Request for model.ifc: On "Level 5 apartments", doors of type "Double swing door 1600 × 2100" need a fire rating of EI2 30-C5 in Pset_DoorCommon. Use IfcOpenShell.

First a look at what the model holds.

```python
import ifcopenshell
import ifcopenshell.util.element

model = ifcopenshell.open("model.ifc")
print(model.schema)
storey = next(s for s in model.by_type("IfcBuildingStorey") if s.Name == "Level 5 apartments")
doors = [e for e in ifcopenshell.util.element.get_decomposition(storey) if e.is_a("IfcDoor")]
seen = {}
for e in doors:
    element_type = ifcopenshell.util.element.get_type(e)
    key = (element_type.Name if element_type != e and element_type else None, ifcopenshell.util.element.get_pset(e, "Pset_DoorCommon", "FireRating"))
    seen[key] = seen.get(key, 0) + 1
for (name, value), count in sorted(seen.items(), key=str):
    print(count, "x", name, "|", value)
```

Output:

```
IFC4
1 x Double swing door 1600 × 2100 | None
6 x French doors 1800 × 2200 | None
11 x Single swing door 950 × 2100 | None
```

```python
import ifcopenshell
import ifcopenshell.api.pset
import ifcopenshell.util.element

model = ifcopenshell.open("model.ifc")

storey = next(s for s in model.by_type("IfcBuildingStorey") if s.Name == "Level 5 apartments")
doors = [e for e in ifcopenshell.util.element.get_decomposition(storey) if e.is_a("IfcDoor")]

count = 0
for e in doors:
    element_type = ifcopenshell.util.element.get_type(e)
    if element_type in (None, e) or element_type.Name != "Double swing door 1600 × 2100":
        continue
    # add_pset returns the element's existing set when there is one.
    pset = ifcopenshell.api.pset.add_pset(model, product=e, name="Pset_DoorCommon")
    ifcopenshell.api.pset.edit_pset(model, pset=pset, properties={"FireRating": "EI2 30-C5"})
    count += 1

print(count, "doors updated")

model.write("model_v2.ifc")
```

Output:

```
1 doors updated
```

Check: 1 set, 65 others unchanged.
